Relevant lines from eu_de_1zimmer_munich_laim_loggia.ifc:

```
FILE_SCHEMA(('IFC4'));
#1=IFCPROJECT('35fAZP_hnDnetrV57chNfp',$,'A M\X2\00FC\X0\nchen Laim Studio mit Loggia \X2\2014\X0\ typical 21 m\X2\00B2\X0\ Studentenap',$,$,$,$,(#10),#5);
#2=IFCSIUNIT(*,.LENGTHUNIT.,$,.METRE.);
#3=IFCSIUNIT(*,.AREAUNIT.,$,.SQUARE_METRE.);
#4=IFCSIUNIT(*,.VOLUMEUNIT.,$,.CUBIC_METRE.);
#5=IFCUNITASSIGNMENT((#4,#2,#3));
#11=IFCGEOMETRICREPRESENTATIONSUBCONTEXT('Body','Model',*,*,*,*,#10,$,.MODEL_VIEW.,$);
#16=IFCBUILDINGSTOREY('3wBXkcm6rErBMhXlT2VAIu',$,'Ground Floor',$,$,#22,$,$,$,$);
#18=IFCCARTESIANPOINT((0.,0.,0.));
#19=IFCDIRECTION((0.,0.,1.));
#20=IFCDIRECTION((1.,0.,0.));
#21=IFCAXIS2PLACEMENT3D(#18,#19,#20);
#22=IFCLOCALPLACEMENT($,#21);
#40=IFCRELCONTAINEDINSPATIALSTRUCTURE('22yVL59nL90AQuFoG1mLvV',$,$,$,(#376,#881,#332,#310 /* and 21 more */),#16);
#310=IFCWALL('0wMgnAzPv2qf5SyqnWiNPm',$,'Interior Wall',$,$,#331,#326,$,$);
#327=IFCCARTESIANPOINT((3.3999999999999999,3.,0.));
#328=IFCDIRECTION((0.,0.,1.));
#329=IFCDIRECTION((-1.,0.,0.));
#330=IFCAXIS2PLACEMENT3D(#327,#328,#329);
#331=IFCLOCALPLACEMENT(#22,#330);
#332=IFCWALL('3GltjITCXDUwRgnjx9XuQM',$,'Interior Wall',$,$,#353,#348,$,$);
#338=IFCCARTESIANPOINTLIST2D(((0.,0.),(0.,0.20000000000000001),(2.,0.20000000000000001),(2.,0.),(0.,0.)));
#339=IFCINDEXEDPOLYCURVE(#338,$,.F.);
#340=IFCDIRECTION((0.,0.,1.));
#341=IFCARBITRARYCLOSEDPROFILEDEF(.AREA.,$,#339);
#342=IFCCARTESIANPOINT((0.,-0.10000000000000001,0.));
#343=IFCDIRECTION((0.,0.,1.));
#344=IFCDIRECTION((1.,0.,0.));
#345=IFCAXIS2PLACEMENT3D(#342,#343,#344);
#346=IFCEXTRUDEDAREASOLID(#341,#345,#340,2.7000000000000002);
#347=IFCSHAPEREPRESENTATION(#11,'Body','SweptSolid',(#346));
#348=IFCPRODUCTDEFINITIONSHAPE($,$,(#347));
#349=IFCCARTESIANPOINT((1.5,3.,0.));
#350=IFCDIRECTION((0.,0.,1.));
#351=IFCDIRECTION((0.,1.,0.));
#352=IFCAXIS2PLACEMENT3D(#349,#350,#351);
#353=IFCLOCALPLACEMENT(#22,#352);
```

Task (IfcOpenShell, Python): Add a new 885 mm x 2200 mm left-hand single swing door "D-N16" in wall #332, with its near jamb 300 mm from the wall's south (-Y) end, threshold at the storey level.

```python
import numpy as np
import ifcopenshell
import ifcopenshell.api.feature
import ifcopenshell.api.geometry
import ifcopenshell.api.root
import ifcopenshell.api.spatial
import ifcopenshell.geom
import ifcopenshell.util.element
import ifcopenshell.util.placement
import ifcopenshell.util.representation
import ifcopenshell.util.shape
import ifcopenshell.util.unit

model = ifcopenshell.open("eu_de_1zimmer_munich_laim_loggia.ifc")
unit_scale = ifcopenshell.util.unit.calculate_unit_scale(model)
settings = ifcopenshell.geom.settings()


def volume(element):
    """Net volume in cubic metres, openings subtracted."""
    shape = ifcopenshell.geom.create_shape(settings, element)
    return ifcopenshell.util.shape.get_volume(shape.geometry)


wall = model.by_guid("3GltjITCXDUwRgnjx9XuQM")
storey = ifcopenshell.util.element.get_container(wall, ifc_class="IfcBuildingStorey")
context = ifcopenshell.util.representation.get_context(model, "Model", "Body", "MODEL_VIEW")
before = volume(wall)

width, height, from_end, sill = 0.885, 2.2, 0.3, 0.0  # metres

# The wall runs along its own X axis, and the end named is its -X end.
wall_shape = ifcopenshell.geom.create_shape(settings, wall)
x, y, z = ifcopenshell.util.shape.get_vertices(wall_shape.geometry).T
start = x.min() + from_end
face, thickness = float(y.min()), float(y.max() - y.min())
wall_matrix = ifcopenshell.util.placement.get_local_placement(wall.ObjectPlacement)
level = ifcopenshell.util.placement.get_local_placement(storey.ObjectPlacement)[2, 3]


def in_wall(x, y):
    """Placement at x, y metres in the wall's axes, at sill height."""
    matrix = wall_matrix.copy()
    matrix[:, 3] = wall_matrix @ np.array([x / unit_scale, y / unit_scale, 0.0, 1.0])
    matrix[2, 3] = level + sill / unit_scale
    return matrix


# Opening: a box that overshoots both wall faces by 50 mm.
opening = ifcopenshell.api.root.create_entity(model, ifc_class="IfcOpeningElement", predefined_type="OPENING")
box = ifcopenshell.api.geometry.add_wall_representation(
    model, context=context, length=width, height=height, thickness=thickness + 0.1
)
ifcopenshell.api.geometry.assign_representation(model, product=opening, representation=box)
ifcopenshell.api.geometry.edit_object_placement(model, product=opening, matrix=in_wall(start, face - 0.05), is_si=False)
ifcopenshell.api.feature.add_feature(model, feature=opening, element=wall)

door = ifcopenshell.api.root.create_entity(model, ifc_class="IfcDoor", name="D-N16", predefined_type="DOOR")
door.OverallWidth, door.OverallHeight = width / unit_scale, height / unit_scale
door.OperationType = "SINGLE_SWING_LEFT"
body = ifcopenshell.api.geometry.add_door_representation(
    model,
    context=context,
    overall_width=door.OverallWidth,
    overall_height=door.OverallHeight,
    operation_type="SINGLE_SWING_LEFT",
    lining_properties={"LiningDepth": thickness / unit_scale, "ThresholdDepth": thickness / unit_scale},
)
ifcopenshell.api.geometry.assign_representation(model, product=door, representation=body)
ifcopenshell.api.spatial.assign_container(model, products=[door], relating_structure=storey)
ifcopenshell.api.feature.add_filling(model, opening=opening, element=door)

# The lining spans the wall, so the door starts at the wall face.
ifcopenshell.api.geometry.edit_object_placement(model, product=door, matrix=in_wall(start, face), is_si=False)

after = volume(wall)

print(f"wall volume {before:.3f} -> {after:.3f} m3")

model.write("eu_de_1zimmer_munich_laim_loggia_edited.ifc")
```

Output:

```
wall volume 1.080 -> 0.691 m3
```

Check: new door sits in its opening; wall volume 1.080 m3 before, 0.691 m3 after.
